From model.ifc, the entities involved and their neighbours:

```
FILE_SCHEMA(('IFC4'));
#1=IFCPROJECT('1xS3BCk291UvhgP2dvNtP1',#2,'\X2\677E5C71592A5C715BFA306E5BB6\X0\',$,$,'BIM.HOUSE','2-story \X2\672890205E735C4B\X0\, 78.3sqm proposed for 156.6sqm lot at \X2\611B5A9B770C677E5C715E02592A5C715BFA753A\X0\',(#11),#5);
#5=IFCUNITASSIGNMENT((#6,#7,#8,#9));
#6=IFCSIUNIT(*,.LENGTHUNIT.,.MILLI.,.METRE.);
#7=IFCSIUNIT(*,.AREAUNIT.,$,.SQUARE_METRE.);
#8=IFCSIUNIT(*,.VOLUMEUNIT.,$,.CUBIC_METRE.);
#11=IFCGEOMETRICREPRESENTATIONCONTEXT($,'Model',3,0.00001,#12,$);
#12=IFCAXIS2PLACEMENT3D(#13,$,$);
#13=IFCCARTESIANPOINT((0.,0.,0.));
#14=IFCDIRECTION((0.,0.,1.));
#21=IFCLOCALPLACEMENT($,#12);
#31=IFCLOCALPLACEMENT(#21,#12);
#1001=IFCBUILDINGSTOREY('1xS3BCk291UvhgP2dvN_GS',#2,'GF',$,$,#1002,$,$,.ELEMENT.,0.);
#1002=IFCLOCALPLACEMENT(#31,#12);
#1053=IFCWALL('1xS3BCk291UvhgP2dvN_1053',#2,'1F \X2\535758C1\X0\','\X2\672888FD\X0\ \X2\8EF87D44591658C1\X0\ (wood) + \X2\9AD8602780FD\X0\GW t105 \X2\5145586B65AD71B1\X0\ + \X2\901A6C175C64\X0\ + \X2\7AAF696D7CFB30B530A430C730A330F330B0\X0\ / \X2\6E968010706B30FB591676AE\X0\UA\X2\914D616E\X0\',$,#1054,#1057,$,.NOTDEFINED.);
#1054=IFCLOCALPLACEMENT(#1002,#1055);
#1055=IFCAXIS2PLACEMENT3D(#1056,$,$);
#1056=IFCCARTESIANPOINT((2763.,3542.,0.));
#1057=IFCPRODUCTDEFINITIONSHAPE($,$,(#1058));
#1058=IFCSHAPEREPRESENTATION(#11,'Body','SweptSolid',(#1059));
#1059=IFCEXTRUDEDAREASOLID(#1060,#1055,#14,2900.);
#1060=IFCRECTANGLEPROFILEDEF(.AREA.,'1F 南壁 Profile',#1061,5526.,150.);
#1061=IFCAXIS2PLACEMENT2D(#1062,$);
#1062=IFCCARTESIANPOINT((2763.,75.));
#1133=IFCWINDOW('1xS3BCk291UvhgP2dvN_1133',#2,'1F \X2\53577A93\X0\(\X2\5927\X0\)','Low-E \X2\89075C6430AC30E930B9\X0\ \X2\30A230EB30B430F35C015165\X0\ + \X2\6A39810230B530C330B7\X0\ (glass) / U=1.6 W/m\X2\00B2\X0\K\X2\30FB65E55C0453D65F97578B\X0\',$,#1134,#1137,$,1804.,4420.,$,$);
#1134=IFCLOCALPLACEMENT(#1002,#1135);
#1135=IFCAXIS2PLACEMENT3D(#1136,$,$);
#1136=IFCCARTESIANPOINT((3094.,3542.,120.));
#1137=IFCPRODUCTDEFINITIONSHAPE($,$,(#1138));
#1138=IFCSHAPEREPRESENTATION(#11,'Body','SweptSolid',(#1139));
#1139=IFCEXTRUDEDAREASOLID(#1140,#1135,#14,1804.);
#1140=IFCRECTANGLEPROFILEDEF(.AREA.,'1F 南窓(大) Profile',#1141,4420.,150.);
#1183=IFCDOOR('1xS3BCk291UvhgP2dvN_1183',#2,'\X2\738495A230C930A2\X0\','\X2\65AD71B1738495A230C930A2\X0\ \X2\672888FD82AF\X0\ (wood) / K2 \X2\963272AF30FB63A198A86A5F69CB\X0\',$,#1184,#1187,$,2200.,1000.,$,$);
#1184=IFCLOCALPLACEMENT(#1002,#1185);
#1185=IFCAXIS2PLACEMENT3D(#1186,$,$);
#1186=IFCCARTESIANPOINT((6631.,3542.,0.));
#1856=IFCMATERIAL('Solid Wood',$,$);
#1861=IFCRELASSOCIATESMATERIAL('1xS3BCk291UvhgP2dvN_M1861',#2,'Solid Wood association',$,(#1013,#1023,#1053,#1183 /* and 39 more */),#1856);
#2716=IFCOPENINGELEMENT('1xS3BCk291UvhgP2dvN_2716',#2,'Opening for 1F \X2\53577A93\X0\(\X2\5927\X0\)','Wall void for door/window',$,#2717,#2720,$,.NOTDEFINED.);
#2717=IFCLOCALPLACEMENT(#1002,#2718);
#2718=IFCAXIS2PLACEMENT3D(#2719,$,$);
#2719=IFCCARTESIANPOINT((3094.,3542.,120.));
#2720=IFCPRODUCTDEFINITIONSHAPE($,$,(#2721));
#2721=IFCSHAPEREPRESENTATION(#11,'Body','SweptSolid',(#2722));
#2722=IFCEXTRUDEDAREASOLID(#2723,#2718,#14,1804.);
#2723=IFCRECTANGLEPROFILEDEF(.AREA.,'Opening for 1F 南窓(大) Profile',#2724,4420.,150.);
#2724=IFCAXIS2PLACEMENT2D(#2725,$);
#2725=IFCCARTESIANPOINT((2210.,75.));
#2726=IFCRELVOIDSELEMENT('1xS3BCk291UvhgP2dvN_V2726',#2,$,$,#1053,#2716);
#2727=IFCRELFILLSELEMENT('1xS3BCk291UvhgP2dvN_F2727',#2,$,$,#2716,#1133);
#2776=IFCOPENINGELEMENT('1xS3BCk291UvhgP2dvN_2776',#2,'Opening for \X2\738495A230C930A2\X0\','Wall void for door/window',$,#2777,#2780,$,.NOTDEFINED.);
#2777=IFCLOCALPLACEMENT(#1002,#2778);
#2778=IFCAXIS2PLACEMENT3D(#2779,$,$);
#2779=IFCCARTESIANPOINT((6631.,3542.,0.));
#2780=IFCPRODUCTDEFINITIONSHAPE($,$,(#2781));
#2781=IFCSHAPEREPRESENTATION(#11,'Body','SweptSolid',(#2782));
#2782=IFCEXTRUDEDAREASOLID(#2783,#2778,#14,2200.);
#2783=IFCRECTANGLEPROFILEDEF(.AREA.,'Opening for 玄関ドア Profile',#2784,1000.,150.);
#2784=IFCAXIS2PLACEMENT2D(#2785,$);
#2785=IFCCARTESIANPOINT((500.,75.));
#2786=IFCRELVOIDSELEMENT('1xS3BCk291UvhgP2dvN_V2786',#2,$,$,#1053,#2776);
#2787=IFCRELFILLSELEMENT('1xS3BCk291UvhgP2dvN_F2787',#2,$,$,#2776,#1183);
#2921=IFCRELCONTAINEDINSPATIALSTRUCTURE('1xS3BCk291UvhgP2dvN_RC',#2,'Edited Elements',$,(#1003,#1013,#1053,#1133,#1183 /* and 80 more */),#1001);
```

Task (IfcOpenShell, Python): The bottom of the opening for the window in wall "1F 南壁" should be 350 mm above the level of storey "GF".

```python
import numpy as np
import ifcopenshell
import ifcopenshell.api.geometry
import ifcopenshell.geom
import ifcopenshell.util.element
import ifcopenshell.util.placement
import ifcopenshell.util.shape
import ifcopenshell.util.unit

model = ifcopenshell.open("model.ifc")
unit_scale = ifcopenshell.util.unit.calculate_unit_scale(model)

window = model.by_guid("1xS3BCk291UvhgP2dvN_1133")
opening = window.FillsVoids[0].RelatingOpeningElement
storey = ifcopenshell.util.element.get_container(window, ifc_class="IfcBuildingStorey")
level = ifcopenshell.util.placement.get_local_placement(storey.ObjectPlacement)[2, 3]

# The opening's origin need not be at the sill, so measure its lowest point.
shape = ifcopenshell.geom.create_shape(ifcopenshell.geom.settings(), opening)
bottom = ifcopenshell.util.shape.get_shape_bottom_elevation(shape, shape.geometry) / unit_scale
dz = level + 0.35 / unit_scale - bottom

shift = np.array([0.0, 0.0, dz])
# The window is not placed relative to its opening, so move both.
for product in (opening, window):
    matrix = ifcopenshell.util.placement.get_local_placement(product.ObjectPlacement)
    matrix[:3, 3] += shift
    ifcopenshell.api.geometry.edit_object_placement(model, product=product, matrix=matrix, is_si=False)

print(f"moved by {dz * unit_scale:+.3f} m")

model.write("model_edited.ifc")
```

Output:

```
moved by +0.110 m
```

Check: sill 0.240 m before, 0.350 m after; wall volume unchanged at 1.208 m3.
